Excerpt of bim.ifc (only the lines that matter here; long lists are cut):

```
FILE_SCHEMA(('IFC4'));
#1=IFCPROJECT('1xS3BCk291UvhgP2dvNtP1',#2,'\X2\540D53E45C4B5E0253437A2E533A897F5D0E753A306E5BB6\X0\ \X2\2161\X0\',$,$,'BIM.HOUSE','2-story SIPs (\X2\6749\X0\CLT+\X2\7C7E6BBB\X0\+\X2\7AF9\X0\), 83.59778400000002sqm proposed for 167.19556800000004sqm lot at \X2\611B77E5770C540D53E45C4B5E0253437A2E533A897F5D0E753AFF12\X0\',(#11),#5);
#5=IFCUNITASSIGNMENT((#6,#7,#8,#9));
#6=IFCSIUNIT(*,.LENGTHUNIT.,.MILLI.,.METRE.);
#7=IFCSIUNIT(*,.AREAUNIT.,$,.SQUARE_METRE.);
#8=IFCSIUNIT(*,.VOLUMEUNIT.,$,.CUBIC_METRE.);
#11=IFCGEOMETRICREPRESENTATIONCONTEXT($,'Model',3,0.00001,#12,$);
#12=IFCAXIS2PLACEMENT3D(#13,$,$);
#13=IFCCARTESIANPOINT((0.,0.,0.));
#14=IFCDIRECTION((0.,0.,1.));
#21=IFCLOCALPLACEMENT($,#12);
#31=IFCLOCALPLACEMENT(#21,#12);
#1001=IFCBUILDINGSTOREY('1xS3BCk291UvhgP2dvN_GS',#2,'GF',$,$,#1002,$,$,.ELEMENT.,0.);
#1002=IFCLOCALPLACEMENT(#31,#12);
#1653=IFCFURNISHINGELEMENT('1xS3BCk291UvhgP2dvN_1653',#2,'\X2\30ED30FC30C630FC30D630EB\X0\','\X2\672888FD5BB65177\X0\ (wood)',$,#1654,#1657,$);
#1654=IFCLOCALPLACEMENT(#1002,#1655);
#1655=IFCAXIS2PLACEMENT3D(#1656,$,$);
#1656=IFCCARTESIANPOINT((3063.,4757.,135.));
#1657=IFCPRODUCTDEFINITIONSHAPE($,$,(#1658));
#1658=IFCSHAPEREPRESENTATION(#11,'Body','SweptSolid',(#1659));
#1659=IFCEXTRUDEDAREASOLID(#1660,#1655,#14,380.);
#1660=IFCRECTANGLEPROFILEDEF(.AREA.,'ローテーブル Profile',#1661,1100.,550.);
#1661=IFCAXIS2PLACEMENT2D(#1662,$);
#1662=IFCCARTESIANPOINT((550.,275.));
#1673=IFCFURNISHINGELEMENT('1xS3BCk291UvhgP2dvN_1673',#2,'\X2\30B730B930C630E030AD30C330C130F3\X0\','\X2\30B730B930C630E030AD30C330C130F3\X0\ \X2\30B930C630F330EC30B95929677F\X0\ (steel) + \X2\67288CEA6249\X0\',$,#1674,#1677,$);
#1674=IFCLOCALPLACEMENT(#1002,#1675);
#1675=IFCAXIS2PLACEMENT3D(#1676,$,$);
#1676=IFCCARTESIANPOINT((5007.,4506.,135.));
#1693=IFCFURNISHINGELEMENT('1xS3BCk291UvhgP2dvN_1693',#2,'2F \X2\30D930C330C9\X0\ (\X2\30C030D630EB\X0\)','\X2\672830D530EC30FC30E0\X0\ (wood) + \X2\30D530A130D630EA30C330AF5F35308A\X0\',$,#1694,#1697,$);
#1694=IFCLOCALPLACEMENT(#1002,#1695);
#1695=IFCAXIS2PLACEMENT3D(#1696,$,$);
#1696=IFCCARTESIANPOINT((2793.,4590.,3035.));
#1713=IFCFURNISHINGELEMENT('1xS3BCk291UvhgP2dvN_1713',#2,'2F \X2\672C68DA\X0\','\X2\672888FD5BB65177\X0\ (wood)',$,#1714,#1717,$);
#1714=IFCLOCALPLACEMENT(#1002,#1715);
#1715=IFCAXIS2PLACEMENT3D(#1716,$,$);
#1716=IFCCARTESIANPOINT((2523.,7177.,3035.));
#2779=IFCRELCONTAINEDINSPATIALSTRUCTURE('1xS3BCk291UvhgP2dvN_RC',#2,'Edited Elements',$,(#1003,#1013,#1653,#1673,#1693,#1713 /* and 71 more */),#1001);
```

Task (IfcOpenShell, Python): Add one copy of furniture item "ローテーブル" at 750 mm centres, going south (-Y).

```python
import numpy as np
import ifcopenshell
import ifcopenshell.api.geometry
import ifcopenshell.api.root
import ifcopenshell.util.element
import ifcopenshell.util.placement
import ifcopenshell.util.unit

model = ifcopenshell.open("bim.ifc")
unit_scale = ifcopenshell.util.unit.calculate_unit_scale(model)


def reuse_history(source, copy):
    """copy_class also copies each property set's owner history, people and application; keep the originals."""
    for rel in copy.IsDefinedBy:
        if rel.is_a("IfcRelDefinesByProperties") and (history := rel.RelatingPropertyDefinition.OwnerHistory):
            rel.RelatingPropertyDefinition.OwnerHistory = source.OwnerHistory
            ifcopenshell.util.element.remove_deep2(model, history)


source = model.by_guid("1xS3BCk291UvhgP2dvN_1653")
base = ifcopenshell.util.placement.get_local_placement(source.ObjectPlacement)
step = np.array([0.0, -1.0, 0.0]) * 0.75 / unit_scale

for i in range(1, 2):
    copy = ifcopenshell.api.root.copy_class(model, product=source)
    copy.Representation = ifcopenshell.util.element.copy_deep(
        model, source.Representation, exclude=["IfcGeometricRepresentationContext", "IfcRepresentationMap"]
    )
    reuse_history(source, copy)
    matrix = base.copy()
    matrix[:3, 3] += i * step
    print("added at", matrix[:3, 3].round(3) + 0.0)
    ifcopenshell.api.geometry.edit_object_placement(model, product=copy, matrix=matrix, is_si=False)

model.write("bim-out.ifc")
```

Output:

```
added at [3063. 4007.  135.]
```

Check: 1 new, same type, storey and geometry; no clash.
